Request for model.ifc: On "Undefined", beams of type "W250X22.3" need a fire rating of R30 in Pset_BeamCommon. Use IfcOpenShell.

First a look at what the model holds.

```python
import ifcopenshell
import ifcopenshell.util.element

model = ifcopenshell.open("model.ifc")
print(model.schema)
storey = next(s for s in model.by_type("IfcBuildingStorey") if s.Name == "Undefined")
beams = [e for e in ifcopenshell.util.element.get_decomposition(storey) if e.is_a("IfcBeam")]
seen = {}
for e in beams:
    element_type = ifcopenshell.util.element.get_type(e)
    key = (element_type.Name if element_type != e and element_type else None, ifcopenshell.util.element.get_pset(e, "Pset_BeamCommon", "FireRating"))
    seen[key] = seen.get(key, 0) + 1
for (name, value), count in sorted(seen.items(), key=str):
    print(count, "x", name, "|", value)
```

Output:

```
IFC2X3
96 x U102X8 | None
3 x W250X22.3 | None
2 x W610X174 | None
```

```python
import ifcopenshell
import ifcopenshell.api.pset
import ifcopenshell.util.element

model = ifcopenshell.open("model.ifc")

storey = next(s for s in model.by_type("IfcBuildingStorey") if s.Name == "Undefined")
beams = [e for e in ifcopenshell.util.element.get_decomposition(storey) if e.is_a("IfcBeam")]

count = 0
for e in beams:
    element_type = ifcopenshell.util.element.get_type(e)
    if element_type in (None, e) or element_type.Name != "W250X22.3":
        continue
    found = ifcopenshell.util.element.get_pset(e, "Pset_BeamCommon", should_inherit=False)
    if found:
        pset = model.by_id(found["id"])
        if len(ifcopenshell.util.element.get_elements_by_pset(pset)) > 1:
            pset = ifcopenshell.api.pset.unshare_pset(model, products=[e], pset=pset)[0]
    else:
        pset = ifcopenshell.api.pset.add_pset(model, product=e, name="Pset_BeamCommon")
    ifcopenshell.api.pset.edit_pset(model, pset=pset, properties={"FireRating": "R30"})
    count += 1

print(count, "beams updated")

model.write("model_updated.ifc")
```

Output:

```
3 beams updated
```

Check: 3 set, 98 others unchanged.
